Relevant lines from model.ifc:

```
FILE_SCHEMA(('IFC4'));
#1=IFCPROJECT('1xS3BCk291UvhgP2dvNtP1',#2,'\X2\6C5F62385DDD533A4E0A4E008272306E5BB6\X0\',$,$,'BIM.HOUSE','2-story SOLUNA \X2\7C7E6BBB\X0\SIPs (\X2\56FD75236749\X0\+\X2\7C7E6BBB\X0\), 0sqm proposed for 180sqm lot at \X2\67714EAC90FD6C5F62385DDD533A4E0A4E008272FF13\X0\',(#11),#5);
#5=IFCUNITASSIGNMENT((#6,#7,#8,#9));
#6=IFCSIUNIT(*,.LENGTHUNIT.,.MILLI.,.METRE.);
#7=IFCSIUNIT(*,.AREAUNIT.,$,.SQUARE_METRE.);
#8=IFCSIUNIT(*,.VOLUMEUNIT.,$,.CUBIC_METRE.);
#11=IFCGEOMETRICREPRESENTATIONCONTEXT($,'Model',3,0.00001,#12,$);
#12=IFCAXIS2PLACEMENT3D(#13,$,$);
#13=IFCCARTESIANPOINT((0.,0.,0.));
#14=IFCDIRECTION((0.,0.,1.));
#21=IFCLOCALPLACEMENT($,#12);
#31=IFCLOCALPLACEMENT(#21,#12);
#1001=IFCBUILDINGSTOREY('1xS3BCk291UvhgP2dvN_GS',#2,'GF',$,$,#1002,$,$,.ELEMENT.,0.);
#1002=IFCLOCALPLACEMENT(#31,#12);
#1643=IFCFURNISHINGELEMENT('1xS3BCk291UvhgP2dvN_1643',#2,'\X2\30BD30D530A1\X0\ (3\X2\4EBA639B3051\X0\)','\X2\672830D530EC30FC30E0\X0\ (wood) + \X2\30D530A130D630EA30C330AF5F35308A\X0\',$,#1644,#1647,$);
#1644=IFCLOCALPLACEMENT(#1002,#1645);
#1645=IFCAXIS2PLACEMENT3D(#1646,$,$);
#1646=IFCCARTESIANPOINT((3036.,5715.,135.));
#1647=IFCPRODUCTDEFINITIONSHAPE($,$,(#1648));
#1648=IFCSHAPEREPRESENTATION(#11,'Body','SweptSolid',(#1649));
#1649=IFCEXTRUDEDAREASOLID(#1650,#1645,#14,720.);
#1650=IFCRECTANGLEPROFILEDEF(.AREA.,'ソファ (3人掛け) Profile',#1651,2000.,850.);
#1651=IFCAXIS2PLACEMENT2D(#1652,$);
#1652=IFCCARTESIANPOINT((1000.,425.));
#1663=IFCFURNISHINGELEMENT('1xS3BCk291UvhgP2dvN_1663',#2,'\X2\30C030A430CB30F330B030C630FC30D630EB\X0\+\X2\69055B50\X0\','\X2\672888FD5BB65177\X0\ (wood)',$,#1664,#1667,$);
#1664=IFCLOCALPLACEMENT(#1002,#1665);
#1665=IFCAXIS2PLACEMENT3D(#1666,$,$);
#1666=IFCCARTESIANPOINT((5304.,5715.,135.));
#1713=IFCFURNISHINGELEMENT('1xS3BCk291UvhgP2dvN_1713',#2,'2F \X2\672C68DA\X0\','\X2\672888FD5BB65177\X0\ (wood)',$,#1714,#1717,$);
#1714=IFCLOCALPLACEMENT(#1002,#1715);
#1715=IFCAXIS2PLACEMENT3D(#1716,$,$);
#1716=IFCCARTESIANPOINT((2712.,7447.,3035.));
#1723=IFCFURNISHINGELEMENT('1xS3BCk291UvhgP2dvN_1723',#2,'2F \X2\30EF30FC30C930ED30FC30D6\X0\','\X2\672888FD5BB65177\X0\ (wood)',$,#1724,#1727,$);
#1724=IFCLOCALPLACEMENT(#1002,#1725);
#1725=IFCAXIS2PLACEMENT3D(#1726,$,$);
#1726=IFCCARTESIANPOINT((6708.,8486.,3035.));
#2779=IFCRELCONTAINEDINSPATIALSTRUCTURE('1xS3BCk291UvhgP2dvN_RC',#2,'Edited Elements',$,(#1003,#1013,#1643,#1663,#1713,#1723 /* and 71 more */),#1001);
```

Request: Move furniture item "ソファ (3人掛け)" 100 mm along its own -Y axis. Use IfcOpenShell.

```python
import ifcopenshell
import ifcopenshell.api.geometry
import ifcopenshell.util.placement

model = ifcopenshell.open("model.ifc")

item = model.by_id(1643)
matrix = ifcopenshell.util.placement.get_local_placement(item.ObjectPlacement)
matrix[:3, 3] -= matrix[:3, 1] * 100.0
ifcopenshell.api.geometry.edit_object_placement(model, product=item, matrix=matrix, is_si=False)

print(ifcopenshell.util.placement.get_local_placement(item.ObjectPlacement).round(3) + 0.0)

model.write("model_updated.ifc")
```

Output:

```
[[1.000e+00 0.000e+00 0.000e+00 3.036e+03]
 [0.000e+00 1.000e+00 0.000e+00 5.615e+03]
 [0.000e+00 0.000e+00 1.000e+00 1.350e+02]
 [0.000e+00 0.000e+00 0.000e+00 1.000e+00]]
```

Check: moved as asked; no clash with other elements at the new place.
